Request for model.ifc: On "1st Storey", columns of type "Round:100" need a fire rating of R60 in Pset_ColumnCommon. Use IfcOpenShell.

First a look at what the model holds.

```python
import ifcopenshell
import ifcopenshell.util.element

model = ifcopenshell.open("model.ifc")
print(model.schema)
storey = next(s for s in model.by_type("IfcBuildingStorey") if s.Name == "1st Storey")
columns = [e for e in ifcopenshell.util.element.get_decomposition(storey) if e.is_a("IfcColumn")]
seen = {}
for e in columns:
    element_type = ifcopenshell.util.element.get_type(e)
    key = (element_type.Name if element_type != e and element_type else None, ifcopenshell.util.element.get_pset(e, "Pset_ColumnCommon", "FireRating"))
    seen[key] = seen.get(key, 0) + 1
for (name, value), count in sorted(seen.items(), key=str):
    print(count, "x", name, "|", value)
```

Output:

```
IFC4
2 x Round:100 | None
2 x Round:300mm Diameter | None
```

```python
import ifcopenshell
import ifcopenshell.api.pset
import ifcopenshell.util.element

model = ifcopenshell.open("model.ifc")

storey = next(s for s in model.by_type("IfcBuildingStorey") if s.Name == "1st Storey")
columns = [e for e in ifcopenshell.util.element.get_decomposition(storey) if e.is_a("IfcColumn")]

count = 0
for e in columns:
    element_type = ifcopenshell.util.element.get_type(e)
    if element_type in (None, e) or element_type.Name != "Round:100":
        continue
    # add_pset returns the element's existing set when there is one.
    pset = ifcopenshell.api.pset.add_pset(model, product=e, name="Pset_ColumnCommon")
    ifcopenshell.api.pset.edit_pset(model, pset=pset, properties={"FireRating": "R60"})
    count += 1

print(count, "columns updated")

model.write("model_v2.ifc")
```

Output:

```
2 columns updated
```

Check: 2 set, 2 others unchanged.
